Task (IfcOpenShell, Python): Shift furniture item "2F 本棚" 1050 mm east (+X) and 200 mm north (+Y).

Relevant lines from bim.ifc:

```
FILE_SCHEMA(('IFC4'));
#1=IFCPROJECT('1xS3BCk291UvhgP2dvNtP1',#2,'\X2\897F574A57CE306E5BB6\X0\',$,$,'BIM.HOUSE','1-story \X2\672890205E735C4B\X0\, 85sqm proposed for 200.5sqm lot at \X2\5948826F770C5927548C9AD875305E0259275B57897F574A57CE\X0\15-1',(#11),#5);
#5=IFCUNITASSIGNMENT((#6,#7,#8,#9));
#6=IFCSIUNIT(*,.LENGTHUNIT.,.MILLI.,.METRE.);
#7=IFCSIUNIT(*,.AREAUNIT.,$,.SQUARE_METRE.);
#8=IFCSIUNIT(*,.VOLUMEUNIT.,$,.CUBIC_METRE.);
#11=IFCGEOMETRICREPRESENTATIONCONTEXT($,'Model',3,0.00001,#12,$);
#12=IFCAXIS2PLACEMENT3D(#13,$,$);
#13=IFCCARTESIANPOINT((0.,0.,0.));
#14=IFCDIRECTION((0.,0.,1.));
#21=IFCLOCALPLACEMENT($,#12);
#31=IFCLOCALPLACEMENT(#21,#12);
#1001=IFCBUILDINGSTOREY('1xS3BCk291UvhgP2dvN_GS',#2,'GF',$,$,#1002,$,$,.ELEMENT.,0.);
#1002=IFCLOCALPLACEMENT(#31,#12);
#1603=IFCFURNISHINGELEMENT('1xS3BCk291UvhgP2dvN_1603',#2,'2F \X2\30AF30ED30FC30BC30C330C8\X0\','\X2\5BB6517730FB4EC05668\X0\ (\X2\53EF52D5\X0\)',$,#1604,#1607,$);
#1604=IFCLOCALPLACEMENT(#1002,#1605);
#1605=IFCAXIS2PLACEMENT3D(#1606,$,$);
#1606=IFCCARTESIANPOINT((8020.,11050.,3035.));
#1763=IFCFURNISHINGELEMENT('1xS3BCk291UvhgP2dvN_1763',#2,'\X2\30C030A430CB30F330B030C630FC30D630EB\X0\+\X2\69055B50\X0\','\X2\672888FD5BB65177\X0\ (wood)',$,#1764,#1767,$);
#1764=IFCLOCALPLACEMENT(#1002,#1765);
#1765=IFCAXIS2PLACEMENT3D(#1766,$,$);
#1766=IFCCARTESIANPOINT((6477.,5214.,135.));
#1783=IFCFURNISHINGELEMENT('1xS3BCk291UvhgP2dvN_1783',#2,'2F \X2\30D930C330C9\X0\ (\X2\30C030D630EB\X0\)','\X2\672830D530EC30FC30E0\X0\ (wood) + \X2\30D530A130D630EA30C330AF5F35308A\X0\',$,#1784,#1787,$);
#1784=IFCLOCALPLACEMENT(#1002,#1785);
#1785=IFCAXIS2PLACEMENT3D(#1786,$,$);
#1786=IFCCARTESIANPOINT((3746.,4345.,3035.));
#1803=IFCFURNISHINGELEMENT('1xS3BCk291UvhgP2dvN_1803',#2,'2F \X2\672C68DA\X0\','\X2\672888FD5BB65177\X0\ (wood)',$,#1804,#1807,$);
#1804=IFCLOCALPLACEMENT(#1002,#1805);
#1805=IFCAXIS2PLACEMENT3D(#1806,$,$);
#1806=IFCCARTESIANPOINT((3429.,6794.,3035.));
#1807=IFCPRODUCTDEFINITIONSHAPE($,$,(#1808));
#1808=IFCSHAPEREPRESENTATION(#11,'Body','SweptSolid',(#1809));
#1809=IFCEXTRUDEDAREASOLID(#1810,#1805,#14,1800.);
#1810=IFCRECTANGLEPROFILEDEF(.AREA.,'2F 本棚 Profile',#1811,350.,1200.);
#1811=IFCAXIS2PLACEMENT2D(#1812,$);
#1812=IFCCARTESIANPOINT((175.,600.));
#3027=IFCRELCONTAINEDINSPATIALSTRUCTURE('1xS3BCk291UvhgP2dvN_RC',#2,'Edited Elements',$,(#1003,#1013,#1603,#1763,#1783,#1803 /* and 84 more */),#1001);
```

```python
import ifcopenshell
import ifcopenshell.api.geometry
import ifcopenshell.util.placement
import ifcopenshell.util.unit

model = ifcopenshell.open("bim.ifc")
unit_scale = ifcopenshell.util.unit.calculate_unit_scale(model)

item = model.by_id(1803)
matrix = ifcopenshell.util.placement.get_local_placement(item.ObjectPlacement)
matrix[0, 3] += 1.05 / unit_scale
matrix[1, 3] += 0.2 / unit_scale
ifcopenshell.api.geometry.edit_object_placement(model, product=item, matrix=matrix, is_si=False)

print(ifcopenshell.util.placement.get_local_placement(item.ObjectPlacement).round(3) + 0.0)

model.write("bim-out.ifc")
```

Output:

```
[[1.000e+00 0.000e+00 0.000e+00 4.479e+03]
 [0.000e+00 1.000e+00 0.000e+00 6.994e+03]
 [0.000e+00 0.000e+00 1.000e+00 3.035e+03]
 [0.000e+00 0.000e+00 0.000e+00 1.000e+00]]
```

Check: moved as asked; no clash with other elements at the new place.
